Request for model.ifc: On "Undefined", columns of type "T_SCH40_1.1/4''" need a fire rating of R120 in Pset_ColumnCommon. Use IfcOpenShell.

First a look at what the model holds.

```python
import ifcopenshell
import ifcopenshell.util.element

model = ifcopenshell.open("model.ifc")
print(model.schema)
storey = next(s for s in model.by_type("IfcBuildingStorey") if s.Name == "Undefined")
columns = [e for e in ifcopenshell.util.element.get_decomposition(storey) if e.is_a("IfcColumn")]
seen = {}
for e in columns:
    element_type = ifcopenshell.util.element.get_type(e)
    key = (element_type.Name if element_type != e and element_type else None, ifcopenshell.util.element.get_pset(e, "Pset_ColumnCommon", "FireRating"))
    seen[key] = seen.get(key, 0) + 1
for (name, value), count in sorted(seen.items(), key=str):
    print(count, "x", name, "|", value)
```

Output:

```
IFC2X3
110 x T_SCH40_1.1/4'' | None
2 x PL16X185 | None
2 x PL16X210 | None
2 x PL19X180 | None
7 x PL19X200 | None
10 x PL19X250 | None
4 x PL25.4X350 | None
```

```python
import ifcopenshell
import ifcopenshell.api.pset
import ifcopenshell.util.element

model = ifcopenshell.open("model.ifc")

storey = next(s for s in model.by_type("IfcBuildingStorey") if s.Name == "Undefined")
columns = [e for e in ifcopenshell.util.element.get_decomposition(storey) if e.is_a("IfcColumn")]

count = 0
for e in columns:
    element_type = ifcopenshell.util.element.get_type(e)
    if element_type in (None, e) or element_type.Name != "T_SCH40_1.1/4''":
        continue
    # add_pset returns the element's existing set when there is one.
    pset = ifcopenshell.api.pset.add_pset(model, product=e, name="Pset_ColumnCommon")
    ifcopenshell.api.pset.edit_pset(model, pset=pset, properties={"FireRating": "R120"})
    count += 1

print(count, "columns updated")

model.write("model_rev.ifc")
```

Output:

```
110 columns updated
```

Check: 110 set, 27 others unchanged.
